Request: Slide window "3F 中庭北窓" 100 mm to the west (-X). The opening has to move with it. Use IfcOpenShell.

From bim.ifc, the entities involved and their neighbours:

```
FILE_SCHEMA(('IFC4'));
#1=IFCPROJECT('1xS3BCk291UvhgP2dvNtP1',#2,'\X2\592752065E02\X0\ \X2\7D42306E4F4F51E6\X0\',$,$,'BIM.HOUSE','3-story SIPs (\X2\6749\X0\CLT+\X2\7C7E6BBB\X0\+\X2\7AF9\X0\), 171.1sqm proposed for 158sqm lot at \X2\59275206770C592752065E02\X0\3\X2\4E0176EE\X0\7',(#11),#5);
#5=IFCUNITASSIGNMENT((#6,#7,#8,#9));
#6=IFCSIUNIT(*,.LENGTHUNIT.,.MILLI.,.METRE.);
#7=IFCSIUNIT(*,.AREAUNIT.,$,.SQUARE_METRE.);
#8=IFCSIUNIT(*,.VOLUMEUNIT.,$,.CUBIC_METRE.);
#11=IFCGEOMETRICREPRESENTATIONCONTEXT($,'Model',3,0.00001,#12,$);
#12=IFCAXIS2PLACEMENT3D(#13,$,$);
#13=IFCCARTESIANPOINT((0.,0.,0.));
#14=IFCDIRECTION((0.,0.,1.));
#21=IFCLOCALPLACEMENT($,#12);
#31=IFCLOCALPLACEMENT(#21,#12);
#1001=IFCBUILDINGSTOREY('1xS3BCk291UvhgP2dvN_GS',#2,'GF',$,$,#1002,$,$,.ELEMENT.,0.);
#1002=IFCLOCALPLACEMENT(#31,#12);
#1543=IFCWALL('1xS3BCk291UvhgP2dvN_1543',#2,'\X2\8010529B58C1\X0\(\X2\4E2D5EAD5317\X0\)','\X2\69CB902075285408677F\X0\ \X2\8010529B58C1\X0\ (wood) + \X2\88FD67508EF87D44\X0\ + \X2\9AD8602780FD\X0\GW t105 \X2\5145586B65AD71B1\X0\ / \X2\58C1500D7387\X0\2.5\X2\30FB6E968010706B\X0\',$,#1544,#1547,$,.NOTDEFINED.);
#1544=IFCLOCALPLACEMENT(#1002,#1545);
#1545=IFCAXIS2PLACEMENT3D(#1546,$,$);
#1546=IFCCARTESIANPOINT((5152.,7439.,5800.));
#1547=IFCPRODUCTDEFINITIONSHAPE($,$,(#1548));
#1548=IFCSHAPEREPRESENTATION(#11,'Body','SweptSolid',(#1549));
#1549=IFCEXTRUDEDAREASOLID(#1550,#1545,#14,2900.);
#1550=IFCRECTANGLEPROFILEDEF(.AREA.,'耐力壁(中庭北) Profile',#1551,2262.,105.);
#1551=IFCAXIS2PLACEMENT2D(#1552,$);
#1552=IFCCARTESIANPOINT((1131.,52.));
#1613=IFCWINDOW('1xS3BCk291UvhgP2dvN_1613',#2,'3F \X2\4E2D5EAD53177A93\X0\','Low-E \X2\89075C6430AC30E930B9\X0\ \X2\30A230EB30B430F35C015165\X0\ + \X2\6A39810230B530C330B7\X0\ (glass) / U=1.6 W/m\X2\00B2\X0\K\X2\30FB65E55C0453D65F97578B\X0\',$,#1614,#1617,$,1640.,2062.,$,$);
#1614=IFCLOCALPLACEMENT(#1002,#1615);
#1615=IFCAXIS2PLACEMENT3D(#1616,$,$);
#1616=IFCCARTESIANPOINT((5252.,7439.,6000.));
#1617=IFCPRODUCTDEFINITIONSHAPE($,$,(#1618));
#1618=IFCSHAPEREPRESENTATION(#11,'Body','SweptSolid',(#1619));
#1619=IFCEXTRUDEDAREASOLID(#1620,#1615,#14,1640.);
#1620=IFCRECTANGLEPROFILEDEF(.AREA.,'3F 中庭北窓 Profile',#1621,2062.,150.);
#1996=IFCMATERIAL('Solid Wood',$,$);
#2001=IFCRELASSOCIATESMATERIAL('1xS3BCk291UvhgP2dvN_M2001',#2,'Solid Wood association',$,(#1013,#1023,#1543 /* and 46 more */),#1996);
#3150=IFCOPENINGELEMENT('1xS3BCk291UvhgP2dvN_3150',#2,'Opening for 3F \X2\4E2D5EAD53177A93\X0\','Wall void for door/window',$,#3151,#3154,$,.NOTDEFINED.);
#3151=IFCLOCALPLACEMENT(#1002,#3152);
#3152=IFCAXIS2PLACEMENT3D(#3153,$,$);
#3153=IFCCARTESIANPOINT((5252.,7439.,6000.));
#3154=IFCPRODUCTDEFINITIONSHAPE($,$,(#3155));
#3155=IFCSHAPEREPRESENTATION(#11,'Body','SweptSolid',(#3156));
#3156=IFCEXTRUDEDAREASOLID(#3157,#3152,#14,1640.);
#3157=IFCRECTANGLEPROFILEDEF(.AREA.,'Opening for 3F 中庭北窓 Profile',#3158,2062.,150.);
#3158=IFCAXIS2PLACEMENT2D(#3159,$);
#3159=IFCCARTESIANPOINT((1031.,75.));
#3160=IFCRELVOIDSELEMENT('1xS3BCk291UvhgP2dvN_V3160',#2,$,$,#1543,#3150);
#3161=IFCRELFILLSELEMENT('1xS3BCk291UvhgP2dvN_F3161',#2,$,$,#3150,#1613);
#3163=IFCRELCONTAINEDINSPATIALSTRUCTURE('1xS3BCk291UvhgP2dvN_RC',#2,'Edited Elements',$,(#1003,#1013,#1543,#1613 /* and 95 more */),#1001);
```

```python
import ifcopenshell
import ifcopenshell.api.geometry
import ifcopenshell.util.placement

model = ifcopenshell.open("bim.ifc")

window = model.by_guid("1xS3BCk291UvhgP2dvN_1613")
opening = window.FillsVoids[0].RelatingOpeningElement
wall = opening.VoidsElements[0].RelatingBuildingElement

wall_matrix = ifcopenshell.util.placement.get_local_placement(wall.ObjectPlacement)
shift = wall_matrix[:3, 0] * -100.0
before = ifcopenshell.util.placement.get_local_placement(window.ObjectPlacement)[:3, 3].copy()

# The window is not placed relative to its opening, so move both.
for product in (opening, window):
    matrix = ifcopenshell.util.placement.get_local_placement(product.ObjectPlacement)
    matrix[:3, 3] += shift
    ifcopenshell.api.geometry.edit_object_placement(model, product=product, matrix=matrix, is_si=False)

after = ifcopenshell.util.placement.get_local_placement(window.ObjectPlacement)[:3, 3]
print("window moved by", (after - before).round(3) + 0.0)

model.write("bim_updated.ifc")
```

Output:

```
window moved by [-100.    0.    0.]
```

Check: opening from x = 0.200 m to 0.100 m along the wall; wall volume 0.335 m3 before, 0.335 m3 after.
